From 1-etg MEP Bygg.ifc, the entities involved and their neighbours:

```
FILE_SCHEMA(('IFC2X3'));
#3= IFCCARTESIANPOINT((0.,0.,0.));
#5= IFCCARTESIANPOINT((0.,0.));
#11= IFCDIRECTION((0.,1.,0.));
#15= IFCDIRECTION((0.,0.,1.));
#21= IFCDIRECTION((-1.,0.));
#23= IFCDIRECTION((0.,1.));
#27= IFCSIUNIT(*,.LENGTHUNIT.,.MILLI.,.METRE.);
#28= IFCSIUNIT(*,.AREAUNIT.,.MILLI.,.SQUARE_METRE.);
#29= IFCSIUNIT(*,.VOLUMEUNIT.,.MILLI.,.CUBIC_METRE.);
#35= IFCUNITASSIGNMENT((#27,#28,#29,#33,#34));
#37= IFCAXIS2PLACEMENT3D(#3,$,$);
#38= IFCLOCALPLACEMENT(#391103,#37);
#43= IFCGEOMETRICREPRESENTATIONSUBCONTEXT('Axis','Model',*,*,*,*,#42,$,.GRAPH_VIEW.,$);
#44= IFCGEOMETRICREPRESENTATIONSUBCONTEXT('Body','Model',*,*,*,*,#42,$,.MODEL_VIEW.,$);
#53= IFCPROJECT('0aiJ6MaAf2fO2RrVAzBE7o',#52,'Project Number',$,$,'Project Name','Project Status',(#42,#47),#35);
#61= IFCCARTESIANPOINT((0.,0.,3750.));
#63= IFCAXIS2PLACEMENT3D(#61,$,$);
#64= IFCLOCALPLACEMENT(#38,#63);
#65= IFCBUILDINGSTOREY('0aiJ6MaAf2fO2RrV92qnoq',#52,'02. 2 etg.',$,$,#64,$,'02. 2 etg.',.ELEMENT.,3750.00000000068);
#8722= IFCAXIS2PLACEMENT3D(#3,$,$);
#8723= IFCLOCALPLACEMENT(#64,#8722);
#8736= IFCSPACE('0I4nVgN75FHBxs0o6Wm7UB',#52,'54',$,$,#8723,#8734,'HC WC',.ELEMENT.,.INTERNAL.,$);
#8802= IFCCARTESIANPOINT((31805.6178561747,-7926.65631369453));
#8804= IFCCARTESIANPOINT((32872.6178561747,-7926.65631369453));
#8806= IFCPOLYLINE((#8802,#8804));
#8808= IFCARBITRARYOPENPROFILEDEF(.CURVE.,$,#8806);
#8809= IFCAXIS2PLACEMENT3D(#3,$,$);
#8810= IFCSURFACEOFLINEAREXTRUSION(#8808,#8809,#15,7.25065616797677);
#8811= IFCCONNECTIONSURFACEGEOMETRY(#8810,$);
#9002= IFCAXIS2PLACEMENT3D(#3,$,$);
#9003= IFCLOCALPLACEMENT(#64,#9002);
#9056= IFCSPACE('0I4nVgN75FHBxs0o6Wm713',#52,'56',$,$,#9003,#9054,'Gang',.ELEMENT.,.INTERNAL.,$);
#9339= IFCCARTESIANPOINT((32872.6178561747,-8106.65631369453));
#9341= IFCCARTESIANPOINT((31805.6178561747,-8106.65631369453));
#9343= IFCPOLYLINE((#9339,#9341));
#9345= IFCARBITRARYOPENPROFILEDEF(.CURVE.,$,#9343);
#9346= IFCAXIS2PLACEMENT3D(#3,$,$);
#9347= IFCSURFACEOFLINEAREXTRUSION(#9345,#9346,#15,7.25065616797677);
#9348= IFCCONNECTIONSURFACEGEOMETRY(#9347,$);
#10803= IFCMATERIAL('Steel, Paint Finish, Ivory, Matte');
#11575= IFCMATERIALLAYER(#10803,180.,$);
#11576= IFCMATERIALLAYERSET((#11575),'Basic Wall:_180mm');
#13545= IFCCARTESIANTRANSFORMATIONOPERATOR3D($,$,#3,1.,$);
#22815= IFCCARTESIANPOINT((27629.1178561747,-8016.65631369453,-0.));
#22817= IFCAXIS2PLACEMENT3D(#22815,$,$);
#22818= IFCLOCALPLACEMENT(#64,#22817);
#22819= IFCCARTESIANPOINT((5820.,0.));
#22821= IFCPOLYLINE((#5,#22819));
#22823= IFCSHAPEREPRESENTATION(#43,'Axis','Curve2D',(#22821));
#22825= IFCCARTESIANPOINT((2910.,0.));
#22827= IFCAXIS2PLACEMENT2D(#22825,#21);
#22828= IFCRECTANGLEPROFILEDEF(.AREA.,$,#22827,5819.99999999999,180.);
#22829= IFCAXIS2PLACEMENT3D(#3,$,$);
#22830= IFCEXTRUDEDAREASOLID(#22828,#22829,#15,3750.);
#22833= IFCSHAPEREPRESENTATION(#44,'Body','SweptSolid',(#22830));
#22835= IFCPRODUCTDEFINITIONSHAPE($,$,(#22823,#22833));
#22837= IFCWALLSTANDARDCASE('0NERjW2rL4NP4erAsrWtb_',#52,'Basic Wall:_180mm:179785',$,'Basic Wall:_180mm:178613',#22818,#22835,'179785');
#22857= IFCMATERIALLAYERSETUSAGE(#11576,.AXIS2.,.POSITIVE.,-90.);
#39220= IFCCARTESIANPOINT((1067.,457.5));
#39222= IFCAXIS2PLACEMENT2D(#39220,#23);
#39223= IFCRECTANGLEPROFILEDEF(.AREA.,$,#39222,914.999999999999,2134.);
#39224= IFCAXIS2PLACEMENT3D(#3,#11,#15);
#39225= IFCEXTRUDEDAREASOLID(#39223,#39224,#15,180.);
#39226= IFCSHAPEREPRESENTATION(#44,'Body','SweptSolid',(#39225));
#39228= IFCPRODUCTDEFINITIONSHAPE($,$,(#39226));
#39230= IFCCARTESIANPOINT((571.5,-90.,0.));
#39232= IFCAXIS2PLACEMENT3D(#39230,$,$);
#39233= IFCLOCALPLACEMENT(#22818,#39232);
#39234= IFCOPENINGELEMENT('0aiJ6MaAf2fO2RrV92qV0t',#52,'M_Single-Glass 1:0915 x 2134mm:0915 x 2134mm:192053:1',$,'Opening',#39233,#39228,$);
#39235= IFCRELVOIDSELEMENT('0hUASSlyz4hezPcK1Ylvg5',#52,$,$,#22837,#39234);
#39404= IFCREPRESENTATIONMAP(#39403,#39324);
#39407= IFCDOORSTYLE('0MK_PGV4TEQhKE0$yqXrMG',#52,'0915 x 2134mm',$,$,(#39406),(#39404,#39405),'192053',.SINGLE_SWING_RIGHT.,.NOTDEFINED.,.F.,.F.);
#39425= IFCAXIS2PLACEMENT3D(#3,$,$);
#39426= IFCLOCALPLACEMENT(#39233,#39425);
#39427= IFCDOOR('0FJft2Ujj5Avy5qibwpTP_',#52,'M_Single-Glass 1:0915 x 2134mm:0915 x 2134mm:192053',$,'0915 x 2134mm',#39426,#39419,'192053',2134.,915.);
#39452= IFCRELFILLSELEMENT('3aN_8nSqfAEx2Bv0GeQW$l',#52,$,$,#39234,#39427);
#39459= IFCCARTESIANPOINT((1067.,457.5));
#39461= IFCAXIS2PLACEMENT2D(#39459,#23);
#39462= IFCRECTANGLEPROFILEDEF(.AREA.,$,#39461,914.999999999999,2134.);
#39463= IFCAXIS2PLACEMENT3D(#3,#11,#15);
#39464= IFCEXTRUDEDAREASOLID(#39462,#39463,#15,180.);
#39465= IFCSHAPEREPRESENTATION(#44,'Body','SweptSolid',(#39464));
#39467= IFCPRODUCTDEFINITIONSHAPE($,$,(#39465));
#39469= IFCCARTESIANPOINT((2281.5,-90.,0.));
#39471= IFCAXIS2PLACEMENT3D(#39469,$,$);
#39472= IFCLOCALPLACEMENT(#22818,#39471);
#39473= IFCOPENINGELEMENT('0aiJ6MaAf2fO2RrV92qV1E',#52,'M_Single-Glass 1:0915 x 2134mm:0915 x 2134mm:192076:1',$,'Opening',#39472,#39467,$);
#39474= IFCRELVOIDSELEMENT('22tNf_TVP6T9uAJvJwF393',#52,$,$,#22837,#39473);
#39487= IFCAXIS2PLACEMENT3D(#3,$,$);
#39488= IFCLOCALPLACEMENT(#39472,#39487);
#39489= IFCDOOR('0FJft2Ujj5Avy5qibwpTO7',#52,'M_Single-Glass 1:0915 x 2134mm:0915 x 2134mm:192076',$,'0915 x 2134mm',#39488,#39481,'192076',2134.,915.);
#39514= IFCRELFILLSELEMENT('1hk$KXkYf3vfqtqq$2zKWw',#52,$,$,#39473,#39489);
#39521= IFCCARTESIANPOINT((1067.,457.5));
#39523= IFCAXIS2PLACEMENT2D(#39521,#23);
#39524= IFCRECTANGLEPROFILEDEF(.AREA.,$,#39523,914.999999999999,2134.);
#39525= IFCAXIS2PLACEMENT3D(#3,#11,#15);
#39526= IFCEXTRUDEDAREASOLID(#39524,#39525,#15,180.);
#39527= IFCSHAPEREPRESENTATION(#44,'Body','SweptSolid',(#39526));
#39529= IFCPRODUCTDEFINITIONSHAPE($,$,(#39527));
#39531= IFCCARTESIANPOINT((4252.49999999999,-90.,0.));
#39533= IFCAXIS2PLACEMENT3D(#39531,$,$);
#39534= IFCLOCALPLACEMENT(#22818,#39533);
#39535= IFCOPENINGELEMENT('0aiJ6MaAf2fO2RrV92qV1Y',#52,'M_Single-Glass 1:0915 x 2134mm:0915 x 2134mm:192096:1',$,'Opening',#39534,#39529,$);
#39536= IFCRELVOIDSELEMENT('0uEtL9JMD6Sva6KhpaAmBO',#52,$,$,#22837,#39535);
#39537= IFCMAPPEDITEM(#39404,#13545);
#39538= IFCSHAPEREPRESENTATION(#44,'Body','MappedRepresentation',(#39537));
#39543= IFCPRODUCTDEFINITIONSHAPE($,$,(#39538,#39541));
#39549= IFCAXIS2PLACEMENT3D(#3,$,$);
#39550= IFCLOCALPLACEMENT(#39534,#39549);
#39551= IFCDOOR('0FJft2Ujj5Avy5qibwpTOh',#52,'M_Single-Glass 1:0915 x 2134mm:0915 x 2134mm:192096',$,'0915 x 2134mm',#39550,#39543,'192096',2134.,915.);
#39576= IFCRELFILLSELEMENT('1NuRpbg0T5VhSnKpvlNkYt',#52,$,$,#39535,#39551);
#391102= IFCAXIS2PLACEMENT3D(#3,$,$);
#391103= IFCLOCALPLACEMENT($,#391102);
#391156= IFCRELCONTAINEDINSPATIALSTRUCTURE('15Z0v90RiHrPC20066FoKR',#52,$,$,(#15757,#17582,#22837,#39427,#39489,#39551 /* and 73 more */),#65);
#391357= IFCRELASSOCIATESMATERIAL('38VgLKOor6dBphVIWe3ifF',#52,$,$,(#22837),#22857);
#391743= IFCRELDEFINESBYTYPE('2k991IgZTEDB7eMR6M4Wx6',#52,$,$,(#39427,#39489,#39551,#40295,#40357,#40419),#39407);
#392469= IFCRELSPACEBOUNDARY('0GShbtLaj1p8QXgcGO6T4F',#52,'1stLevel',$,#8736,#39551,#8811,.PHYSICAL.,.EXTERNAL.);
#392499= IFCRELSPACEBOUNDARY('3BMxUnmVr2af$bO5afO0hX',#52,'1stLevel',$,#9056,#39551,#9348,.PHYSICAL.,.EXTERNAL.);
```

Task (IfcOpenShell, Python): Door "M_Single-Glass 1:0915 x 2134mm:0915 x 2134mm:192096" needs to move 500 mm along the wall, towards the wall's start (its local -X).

```python
import numpy as np
import ifcopenshell
import ifcopenshell.api.geometry
import ifcopenshell.util.placement
import ifcopenshell.util.unit

model = ifcopenshell.open("1-etg MEP Bygg.ifc")
unit_scale = ifcopenshell.util.unit.calculate_unit_scale(model)

door = model.by_guid("0FJft2Ujj5Avy5qibwpTOh")
opening = door.FillsVoids[0].RelatingOpeningElement
wall = opening.VoidsElements[0].RelatingBuildingElement

wall_matrix = ifcopenshell.util.placement.get_local_placement(wall.ObjectPlacement)
shift = wall_matrix[:3, 0] * -0.5 / unit_scale
before = ifcopenshell.util.placement.get_local_placement(door.ObjectPlacement)[:3, 3].copy()

# The door is placed relative to its opening, so it follows when the opening moves.
matrix = ifcopenshell.util.placement.get_local_placement(opening.ObjectPlacement)
matrix[:3, 3] += shift
ifcopenshell.api.geometry.edit_object_placement(
    model, product=opening, matrix=matrix, is_si=False, should_transform_children=True
)

# Space boundary surfaces are stored in each space's coordinates; move them too.
for rel in door.ProvidesBoundaries:
    if not rel.ConnectionGeometry:
        continue
    surface = rel.ConnectionGeometry.SurfaceOnRelatingElement
    space_matrix = ifcopenshell.util.placement.get_local_placement(rel.RelatingSpace.ObjectPlacement)
    point = np.array(surface.Position.Location.Coordinates) + space_matrix[:3, :3].T @ shift
    surface.Position = model.createIfcAxis2Placement3D(
        model.createIfcCartesianPoint(point.tolist()), surface.Position.Axis, surface.Position.RefDirection
    )

after = ifcopenshell.util.placement.get_local_placement(door.ObjectPlacement)[:3, 3]
print("door moved by", (after - before).round(3) + 0.0)

model.write("1-etg MEP Bygg_v2.ifc")
```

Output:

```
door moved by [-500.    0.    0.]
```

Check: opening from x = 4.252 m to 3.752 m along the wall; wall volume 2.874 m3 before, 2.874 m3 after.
